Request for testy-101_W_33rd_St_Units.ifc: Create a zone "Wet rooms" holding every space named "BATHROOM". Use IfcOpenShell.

First a look at what the model holds.

```python
import ifcopenshell

model = ifcopenshell.open("testy-101_W_33rd_St_Units.ifc")
print(model.schema)
seen = {}
for space in model.by_type("IfcSpace"):
    seen[space.LongName] = seen.get(space.LongName, 0) + 1
for name, count in sorted(seen.items(), key=str):
    print(count, "x", name)
print("zones:", [z.Name for z in model.by_type("IfcZone")][:20])
```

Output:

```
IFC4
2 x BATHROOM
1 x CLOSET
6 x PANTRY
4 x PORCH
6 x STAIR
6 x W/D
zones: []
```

```python
import ifcopenshell
import ifcopenshell.api.group
import ifcopenshell.api.root

model = ifcopenshell.open("testy-101_W_33rd_St_Units.ifc")

names = {"BATHROOM"}
spaces = [s for s in model.by_type("IfcSpace") if s.LongName in names]

zone = ifcopenshell.api.root.create_entity(model, ifc_class="IfcZone", name="Wet rooms")
ifcopenshell.api.group.assign_group(model, products=spaces, group=zone)
print(len(spaces), "spaces in", zone.Name)

model.write("testy-101_W_33rd_St_Units-out.ifc")
```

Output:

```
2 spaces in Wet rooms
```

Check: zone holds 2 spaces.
